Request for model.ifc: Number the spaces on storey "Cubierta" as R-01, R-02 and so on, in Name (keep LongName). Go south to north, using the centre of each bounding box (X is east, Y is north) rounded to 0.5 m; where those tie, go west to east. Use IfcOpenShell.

First a look at what the model holds.

```python
import ifcopenshell
import ifcopenshell.util.element
import ifcopenshell.util.placement

model = ifcopenshell.open("model.ifc")
print(model.schema)
storey = next(s for s in model.by_type("IfcBuildingStorey") if s.Name == "Cubierta")
spaces = [e for e in ifcopenshell.util.element.get_decomposition(storey) if e.is_a("IfcSpace")]
for e in sorted(spaces, key=lambda e: e.id()):
    origin = ifcopenshell.util.placement.get_local_placement(e.ObjectPlacement)[:3, 3]
    print(e.id(), e.Name, e.LongName, origin.round(2) + 0.0, sep=" | ")
```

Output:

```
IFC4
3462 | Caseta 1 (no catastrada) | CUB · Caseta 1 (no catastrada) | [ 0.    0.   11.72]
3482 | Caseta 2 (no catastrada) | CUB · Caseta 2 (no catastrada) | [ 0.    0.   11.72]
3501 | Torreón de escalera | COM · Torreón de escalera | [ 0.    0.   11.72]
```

```python
import ifcopenshell
import ifcopenshell.geom
import ifcopenshell.util.element
import ifcopenshell.util.shape

model = ifcopenshell.open("model.ifc")
settings = ifcopenshell.geom.settings()
settings.set("use-world-coords", True)


def centre(element):
    shape = ifcopenshell.geom.create_shape(settings, element)
    return ifcopenshell.util.shape.get_bbox_centroid(shape.geometry)


storey = next(s for s in model.by_type("IfcBuildingStorey") if s.Name == "Cubierta")
spaces = [e for e in ifcopenshell.util.element.get_decomposition(storey) if e.is_a("IfcSpace")]

# Insertion points can sit at a corner or the storey origin, so sort by the geometry (in metres).
centres = {e: centre(e) for e in spaces}
spaces.sort(key=lambda e: (round(centres[e][1] / 0.5), centres[e][0]))

for i, e in enumerate(spaces, start=1):
    number = f"R-{i:02d}"
    e.Name = number
    print(e.id(), number)

model.write("model_rev.ifc")
```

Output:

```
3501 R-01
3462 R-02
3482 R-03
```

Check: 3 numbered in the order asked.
